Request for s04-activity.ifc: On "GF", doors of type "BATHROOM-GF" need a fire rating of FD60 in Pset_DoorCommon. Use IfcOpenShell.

First a look at what the model holds.

```python
import ifcopenshell
import ifcopenshell.util.element

model = ifcopenshell.open("s04-activity.ifc")
print(model.schema)
storey = next(s for s in model.by_type("IfcBuildingStorey") if s.Name == "GF")
doors = [e for e in ifcopenshell.util.element.get_decomposition(storey) if e.is_a("IfcDoor")]
seen = {}
for e in doors:
    element_type = ifcopenshell.util.element.get_type(e)
    key = (element_type.Name if element_type != e and element_type else None, ifcopenshell.util.element.get_pset(e, "Pset_DoorCommon", "FireRating"))
    seen[key] = seen.get(key, 0) + 1
for (name, value), count in sorted(seen.items(), key=str):
    print(count, "x", name, "|", value)
```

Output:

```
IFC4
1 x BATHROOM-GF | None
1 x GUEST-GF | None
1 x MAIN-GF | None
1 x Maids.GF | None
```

```python
import ifcopenshell
import ifcopenshell.api.pset
import ifcopenshell.util.element

model = ifcopenshell.open("s04-activity.ifc")

storey = next(s for s in model.by_type("IfcBuildingStorey") if s.Name == "GF")
doors = [e for e in ifcopenshell.util.element.get_decomposition(storey) if e.is_a("IfcDoor")]

count = 0
for e in doors:
    element_type = ifcopenshell.util.element.get_type(e)
    if element_type in (None, e) or element_type.Name != "BATHROOM-GF":
        continue
    # add_pset returns the element's existing set when there is one.
    pset = ifcopenshell.api.pset.add_pset(model, product=e, name="Pset_DoorCommon")
    ifcopenshell.api.pset.edit_pset(model, pset=pset, properties={"FireRating": "FD60"})
    count += 1

print(count, "doors updated")

model.write("s04-activity_updated.ifc")
```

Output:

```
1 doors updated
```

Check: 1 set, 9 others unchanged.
